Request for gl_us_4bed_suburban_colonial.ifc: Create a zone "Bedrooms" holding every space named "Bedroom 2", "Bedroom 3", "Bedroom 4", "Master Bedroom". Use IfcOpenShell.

First a look at what the model holds.

```python
import ifcopenshell

model = ifcopenshell.open("gl_us_4bed_suburban_colonial.ifc")
print(model.schema)
seen = {}
for space in model.by_type("IfcSpace"):
    seen[space.LongName] = seen.get(space.LongName, 0) + 1
for name, count in sorted(seen.items(), key=str):
    print(count, "x", name)
print("zones:", [z.Name for z in model.by_type("IfcZone")][:20])
```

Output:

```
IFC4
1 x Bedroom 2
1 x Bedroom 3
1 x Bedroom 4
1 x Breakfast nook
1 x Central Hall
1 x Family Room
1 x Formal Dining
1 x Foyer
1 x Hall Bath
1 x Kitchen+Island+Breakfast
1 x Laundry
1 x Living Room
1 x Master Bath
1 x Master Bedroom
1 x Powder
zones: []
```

```python
import ifcopenshell
import ifcopenshell.api.group
import ifcopenshell.api.root

model = ifcopenshell.open("gl_us_4bed_suburban_colonial.ifc")

names = {"Bedroom 2", "Bedroom 3", "Bedroom 4", "Master Bedroom"}
spaces = [s for s in model.by_type("IfcSpace") if s.LongName in names]

zone = ifcopenshell.api.root.create_entity(model, ifc_class="IfcZone", name="Bedrooms")
ifcopenshell.api.group.assign_group(model, products=spaces, group=zone)
print(len(spaces), "spaces in", zone.Name)

model.write("gl_us_4bed_suburban_colonial-out.ifc")
```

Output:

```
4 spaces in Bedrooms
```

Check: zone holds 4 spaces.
